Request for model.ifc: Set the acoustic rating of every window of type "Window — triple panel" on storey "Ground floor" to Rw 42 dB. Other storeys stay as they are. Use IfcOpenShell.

First a look at what the model holds.

```python
import ifcopenshell
import ifcopenshell.util.element

model = ifcopenshell.open("model.ifc")
print(model.schema)
storey = next(s for s in model.by_type("IfcBuildingStorey") if s.Name == "Ground floor")
windows = [e for e in ifcopenshell.util.element.get_decomposition(storey) if e.is_a("IfcWindow")]
seen = {}
for e in windows:
    element_type = ifcopenshell.util.element.get_type(e)
    key = (element_type.Name if element_type != e and element_type else None, ifcopenshell.util.element.get_pset(e, "Pset_WindowCommon", "AcousticRating"))
    seen[key] = seen.get(key, 0) + 1
for (name, value), count in sorted(seen.items(), key=str):
    print(count, "x", name, "|", value)
```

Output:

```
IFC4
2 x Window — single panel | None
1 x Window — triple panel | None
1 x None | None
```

```python
import ifcopenshell
import ifcopenshell.api.pset
import ifcopenshell.util.element

model = ifcopenshell.open("model.ifc")

storey = next(s for s in model.by_type("IfcBuildingStorey") if s.Name == "Ground floor")
windows = [e for e in ifcopenshell.util.element.get_decomposition(storey) if e.is_a("IfcWindow")]

count = 0
for e in windows:
    element_type = ifcopenshell.util.element.get_type(e)
    if element_type in (None, e) or element_type.Name != "Window — triple panel":
        continue
    # add_pset returns the element's existing set when there is one.
    pset = ifcopenshell.api.pset.add_pset(model, product=e, name="Pset_WindowCommon")
    ifcopenshell.api.pset.edit_pset(model, pset=pset, properties={"AcousticRating": "Rw 42 dB"})
    count += 1

print(count, "windows updated")

model.write("model-out.ifc")
```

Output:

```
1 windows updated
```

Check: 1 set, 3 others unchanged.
